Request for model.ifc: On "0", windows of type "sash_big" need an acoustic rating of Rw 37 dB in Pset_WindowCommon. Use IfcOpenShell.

First a look at what the model holds.

```python
import ifcopenshell
import ifcopenshell.util.element

model = ifcopenshell.open("model.ifc")
print(model.schema)
storey = next(s for s in model.by_type("IfcBuildingStorey") if s.Name == "0")
windows = [e for e in ifcopenshell.util.element.get_decomposition(storey) if e.is_a("IfcWindow")]
seen = {}
for e in windows:
    element_type = ifcopenshell.util.element.get_type(e)
    key = (element_type.Name if element_type != e and element_type else None, ifcopenshell.util.element.get_pset(e, "Pset_WindowCommon", "AcousticRating"))
    seen[key] = seen.get(key, 0) + 1
for (name, value), count in sorted(seen.items(), key=str):
    print(count, "x", name, "|", value)
```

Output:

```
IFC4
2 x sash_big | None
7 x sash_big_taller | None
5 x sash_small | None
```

```python
import ifcopenshell
import ifcopenshell.api.pset
import ifcopenshell.util.element

model = ifcopenshell.open("model.ifc")

storey = next(s for s in model.by_type("IfcBuildingStorey") if s.Name == "0")
windows = [e for e in ifcopenshell.util.element.get_decomposition(storey) if e.is_a("IfcWindow")]

count = 0
for e in windows:
    element_type = ifcopenshell.util.element.get_type(e)
    if element_type in (None, e) or element_type.Name != "sash_big":
        continue
    # add_pset returns the element's existing set when there is one.
    pset = ifcopenshell.api.pset.add_pset(model, product=e, name="Pset_WindowCommon")
    ifcopenshell.api.pset.edit_pset(model, pset=pset, properties={"AcousticRating": "Rw 37 dB"})
    count += 1

print(count, "windows updated")

model.write("model-out.ifc")
```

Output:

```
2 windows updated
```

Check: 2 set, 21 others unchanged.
